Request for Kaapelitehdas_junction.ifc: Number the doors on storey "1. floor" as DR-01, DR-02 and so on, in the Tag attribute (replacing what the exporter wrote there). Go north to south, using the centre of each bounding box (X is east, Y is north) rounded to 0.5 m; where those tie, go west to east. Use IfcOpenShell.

First a look at what the model holds.

```python
import ifcopenshell
import ifcopenshell.util.element
import ifcopenshell.util.placement

model = ifcopenshell.open("Kaapelitehdas_junction.ifc")
print(model.schema)
storey = next(s for s in model.by_type("IfcBuildingStorey") if s.Name == "1. floor")
doors = [e for e in ifcopenshell.util.element.get_decomposition(storey) if e.is_a("IfcDoor")]
for e in sorted(doors, key=lambda e: e.id()):
    origin = ifcopenshell.util.placement.get_local_placement(e.ObjectPlacement)[:3, 3]
    print(e.id(), e.Tag, e.Name, origin.round(2) + 0.0, sep=" | ")
```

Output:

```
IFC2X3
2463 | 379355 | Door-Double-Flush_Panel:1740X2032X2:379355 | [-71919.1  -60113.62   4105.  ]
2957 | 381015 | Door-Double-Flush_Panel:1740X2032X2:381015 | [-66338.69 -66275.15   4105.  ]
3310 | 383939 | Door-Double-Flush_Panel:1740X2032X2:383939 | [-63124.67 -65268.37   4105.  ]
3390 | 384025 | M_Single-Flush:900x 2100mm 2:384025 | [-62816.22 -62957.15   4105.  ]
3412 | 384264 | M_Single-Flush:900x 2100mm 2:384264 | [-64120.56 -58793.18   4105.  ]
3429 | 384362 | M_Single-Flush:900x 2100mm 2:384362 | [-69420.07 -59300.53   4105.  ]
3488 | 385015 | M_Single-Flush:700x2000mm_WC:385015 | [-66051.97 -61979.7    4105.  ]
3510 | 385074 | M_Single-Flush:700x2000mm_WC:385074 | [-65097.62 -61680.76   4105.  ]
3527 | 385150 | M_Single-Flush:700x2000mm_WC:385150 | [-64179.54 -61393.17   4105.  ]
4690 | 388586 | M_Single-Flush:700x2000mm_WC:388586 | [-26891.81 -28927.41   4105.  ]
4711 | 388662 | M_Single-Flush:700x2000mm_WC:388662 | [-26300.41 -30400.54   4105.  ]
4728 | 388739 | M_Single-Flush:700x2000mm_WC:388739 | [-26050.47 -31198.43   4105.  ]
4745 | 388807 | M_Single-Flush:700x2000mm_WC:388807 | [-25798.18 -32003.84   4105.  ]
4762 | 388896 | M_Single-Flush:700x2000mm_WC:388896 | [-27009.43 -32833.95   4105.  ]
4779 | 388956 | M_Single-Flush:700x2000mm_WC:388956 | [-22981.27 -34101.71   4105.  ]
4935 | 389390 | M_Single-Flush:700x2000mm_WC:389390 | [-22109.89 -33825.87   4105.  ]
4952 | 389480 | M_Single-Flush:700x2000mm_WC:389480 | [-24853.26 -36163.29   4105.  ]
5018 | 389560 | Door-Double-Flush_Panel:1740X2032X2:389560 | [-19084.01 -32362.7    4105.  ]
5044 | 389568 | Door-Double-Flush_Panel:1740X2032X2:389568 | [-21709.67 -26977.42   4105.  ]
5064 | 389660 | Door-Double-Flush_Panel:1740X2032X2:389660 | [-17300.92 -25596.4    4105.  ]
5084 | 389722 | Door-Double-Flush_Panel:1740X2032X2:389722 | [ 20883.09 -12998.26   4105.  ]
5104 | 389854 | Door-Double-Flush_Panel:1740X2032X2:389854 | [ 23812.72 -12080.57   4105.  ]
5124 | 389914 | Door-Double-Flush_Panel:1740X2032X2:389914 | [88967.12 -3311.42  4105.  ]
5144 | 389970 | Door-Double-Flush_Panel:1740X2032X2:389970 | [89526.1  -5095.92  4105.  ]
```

```python
import ifcopenshell
import ifcopenshell.geom
import ifcopenshell.util.element
import ifcopenshell.util.shape

model = ifcopenshell.open("Kaapelitehdas_junction.ifc")
settings = ifcopenshell.geom.settings()
settings.set("use-world-coords", True)


def centre(element):
    shape = ifcopenshell.geom.create_shape(settings, element)
    return ifcopenshell.util.shape.get_bbox_centroid(shape.geometry)


storey = next(s for s in model.by_type("IfcBuildingStorey") if s.Name == "1. floor")
doors = [e for e in ifcopenshell.util.element.get_decomposition(storey) if e.is_a("IfcDoor")]

# Insertion points can sit at a corner or the storey origin, so sort by the geometry (in metres).
centres = {e: centre(e) for e in doors}
doors.sort(key=lambda e: (-round(centres[e][1] / 0.5), centres[e][0]))

for i, e in enumerate(doors, start=1):
    number = f"DR-{i:02d}"
    e.Tag = number
    print(e.id(), number)

model.write("Kaapelitehdas_junction_updated.ifc")
```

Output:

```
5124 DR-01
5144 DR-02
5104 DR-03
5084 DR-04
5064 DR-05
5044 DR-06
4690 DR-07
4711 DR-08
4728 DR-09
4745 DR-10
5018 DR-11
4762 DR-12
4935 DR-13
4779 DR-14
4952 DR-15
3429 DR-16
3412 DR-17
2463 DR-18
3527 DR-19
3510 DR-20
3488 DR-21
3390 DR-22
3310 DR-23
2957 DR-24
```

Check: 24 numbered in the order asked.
